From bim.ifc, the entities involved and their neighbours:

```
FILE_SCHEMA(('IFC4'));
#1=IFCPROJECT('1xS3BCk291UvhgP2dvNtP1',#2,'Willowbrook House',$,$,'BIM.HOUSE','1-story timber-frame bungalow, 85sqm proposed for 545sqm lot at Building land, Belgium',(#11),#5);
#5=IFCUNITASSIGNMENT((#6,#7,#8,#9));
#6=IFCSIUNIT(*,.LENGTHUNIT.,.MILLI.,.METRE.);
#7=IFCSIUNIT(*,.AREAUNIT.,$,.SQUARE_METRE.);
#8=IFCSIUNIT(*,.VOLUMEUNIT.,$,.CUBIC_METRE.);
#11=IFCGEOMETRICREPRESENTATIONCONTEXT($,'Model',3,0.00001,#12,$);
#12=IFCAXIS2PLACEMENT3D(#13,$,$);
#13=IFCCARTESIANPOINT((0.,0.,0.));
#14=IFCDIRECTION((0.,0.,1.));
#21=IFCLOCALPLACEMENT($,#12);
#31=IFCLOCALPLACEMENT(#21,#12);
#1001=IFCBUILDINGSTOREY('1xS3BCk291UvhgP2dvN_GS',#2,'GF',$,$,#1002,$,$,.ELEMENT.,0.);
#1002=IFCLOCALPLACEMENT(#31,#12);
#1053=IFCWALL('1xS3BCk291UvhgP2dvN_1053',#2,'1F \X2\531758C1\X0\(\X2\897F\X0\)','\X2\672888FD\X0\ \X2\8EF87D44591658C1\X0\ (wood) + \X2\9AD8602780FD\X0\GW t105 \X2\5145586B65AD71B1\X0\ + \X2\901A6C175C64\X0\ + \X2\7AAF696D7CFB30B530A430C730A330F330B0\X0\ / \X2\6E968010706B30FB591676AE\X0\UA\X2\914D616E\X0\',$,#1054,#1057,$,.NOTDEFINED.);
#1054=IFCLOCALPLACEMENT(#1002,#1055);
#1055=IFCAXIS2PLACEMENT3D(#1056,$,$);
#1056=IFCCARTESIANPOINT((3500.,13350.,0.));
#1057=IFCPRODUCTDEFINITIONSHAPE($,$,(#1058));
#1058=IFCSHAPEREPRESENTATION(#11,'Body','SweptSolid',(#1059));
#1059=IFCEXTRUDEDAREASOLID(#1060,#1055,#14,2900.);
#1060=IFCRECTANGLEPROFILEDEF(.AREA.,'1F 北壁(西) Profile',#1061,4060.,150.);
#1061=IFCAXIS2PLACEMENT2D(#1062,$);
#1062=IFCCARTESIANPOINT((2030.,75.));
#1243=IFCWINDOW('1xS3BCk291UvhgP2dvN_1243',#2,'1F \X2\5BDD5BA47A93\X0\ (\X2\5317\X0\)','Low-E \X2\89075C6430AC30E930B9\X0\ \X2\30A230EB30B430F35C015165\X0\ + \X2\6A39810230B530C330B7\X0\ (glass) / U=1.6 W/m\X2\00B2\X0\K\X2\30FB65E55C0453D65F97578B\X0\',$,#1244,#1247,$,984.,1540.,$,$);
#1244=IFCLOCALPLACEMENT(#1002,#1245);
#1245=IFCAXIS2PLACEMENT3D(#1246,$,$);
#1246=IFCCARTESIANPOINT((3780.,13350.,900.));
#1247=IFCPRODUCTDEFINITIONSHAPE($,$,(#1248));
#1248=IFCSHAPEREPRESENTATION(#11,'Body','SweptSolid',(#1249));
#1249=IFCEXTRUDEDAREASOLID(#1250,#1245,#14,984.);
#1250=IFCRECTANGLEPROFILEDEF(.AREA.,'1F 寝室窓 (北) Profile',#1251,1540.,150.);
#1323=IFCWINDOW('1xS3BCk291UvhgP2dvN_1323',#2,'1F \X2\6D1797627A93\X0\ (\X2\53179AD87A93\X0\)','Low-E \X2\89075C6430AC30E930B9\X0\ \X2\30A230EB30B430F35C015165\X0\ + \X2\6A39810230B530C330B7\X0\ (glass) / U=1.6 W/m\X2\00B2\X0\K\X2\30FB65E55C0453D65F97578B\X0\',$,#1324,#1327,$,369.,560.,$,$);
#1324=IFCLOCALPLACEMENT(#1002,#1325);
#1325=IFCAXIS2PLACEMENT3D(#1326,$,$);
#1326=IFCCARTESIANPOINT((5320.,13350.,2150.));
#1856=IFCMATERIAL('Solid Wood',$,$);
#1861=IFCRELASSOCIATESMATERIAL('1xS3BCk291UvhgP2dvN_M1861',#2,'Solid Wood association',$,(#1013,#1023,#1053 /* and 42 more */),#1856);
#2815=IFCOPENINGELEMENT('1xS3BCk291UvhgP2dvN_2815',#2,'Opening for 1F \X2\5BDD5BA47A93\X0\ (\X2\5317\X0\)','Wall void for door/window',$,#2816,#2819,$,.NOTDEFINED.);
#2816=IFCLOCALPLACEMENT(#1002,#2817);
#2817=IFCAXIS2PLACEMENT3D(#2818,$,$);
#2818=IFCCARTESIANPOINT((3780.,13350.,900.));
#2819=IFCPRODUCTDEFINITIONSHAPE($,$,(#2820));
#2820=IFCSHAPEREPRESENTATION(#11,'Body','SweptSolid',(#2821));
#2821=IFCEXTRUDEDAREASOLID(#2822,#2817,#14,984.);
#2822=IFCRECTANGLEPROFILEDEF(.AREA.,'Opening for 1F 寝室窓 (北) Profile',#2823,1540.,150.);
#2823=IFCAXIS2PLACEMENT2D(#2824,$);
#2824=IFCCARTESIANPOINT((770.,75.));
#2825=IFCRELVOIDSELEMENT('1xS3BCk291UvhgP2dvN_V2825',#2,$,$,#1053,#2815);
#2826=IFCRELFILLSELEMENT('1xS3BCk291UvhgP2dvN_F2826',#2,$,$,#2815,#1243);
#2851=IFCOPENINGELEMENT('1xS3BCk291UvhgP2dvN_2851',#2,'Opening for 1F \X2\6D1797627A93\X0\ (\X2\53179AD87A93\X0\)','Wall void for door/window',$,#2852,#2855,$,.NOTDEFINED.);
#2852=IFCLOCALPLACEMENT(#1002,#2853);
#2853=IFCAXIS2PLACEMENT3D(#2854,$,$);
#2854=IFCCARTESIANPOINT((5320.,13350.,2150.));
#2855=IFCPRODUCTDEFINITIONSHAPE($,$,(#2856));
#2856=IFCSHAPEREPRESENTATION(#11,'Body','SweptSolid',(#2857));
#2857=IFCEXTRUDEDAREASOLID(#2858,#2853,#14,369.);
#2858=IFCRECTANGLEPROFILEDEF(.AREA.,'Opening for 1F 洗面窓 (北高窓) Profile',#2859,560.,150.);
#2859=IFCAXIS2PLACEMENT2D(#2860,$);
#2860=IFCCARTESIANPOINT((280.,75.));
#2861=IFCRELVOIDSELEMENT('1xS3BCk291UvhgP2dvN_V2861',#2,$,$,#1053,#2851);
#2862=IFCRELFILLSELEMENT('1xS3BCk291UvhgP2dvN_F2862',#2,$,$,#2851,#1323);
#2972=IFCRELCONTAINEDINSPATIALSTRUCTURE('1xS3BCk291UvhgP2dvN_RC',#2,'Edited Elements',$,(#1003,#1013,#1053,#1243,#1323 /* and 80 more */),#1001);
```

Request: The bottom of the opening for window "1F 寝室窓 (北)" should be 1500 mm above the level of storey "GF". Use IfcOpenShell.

```python
import numpy as np
import ifcopenshell
import ifcopenshell.api.geometry
import ifcopenshell.geom
import ifcopenshell.util.element
import ifcopenshell.util.placement
import ifcopenshell.util.shape
import ifcopenshell.util.unit

model = ifcopenshell.open("bim.ifc")
unit_scale = ifcopenshell.util.unit.calculate_unit_scale(model)

window = model.by_id(1243)
opening = window.FillsVoids[0].RelatingOpeningElement
storey = ifcopenshell.util.element.get_container(window, ifc_class="IfcBuildingStorey")
level = ifcopenshell.util.placement.get_local_placement(storey.ObjectPlacement)[2, 3]

# The opening's origin need not be at the sill, so measure its lowest point.
shape = ifcopenshell.geom.create_shape(ifcopenshell.geom.settings(), opening)
bottom = ifcopenshell.util.shape.get_shape_bottom_elevation(shape, shape.geometry) / unit_scale
dz = level + 1500.0 - bottom

shift = np.array([0.0, 0.0, dz])
# The window is not placed relative to its opening, so move both.
for product in (opening, window):
    matrix = ifcopenshell.util.placement.get_local_placement(product.ObjectPlacement)
    matrix[:3, 3] += shift
    ifcopenshell.api.geometry.edit_object_placement(model, product=product, matrix=matrix, is_si=False)

print(f"moved by {dz * unit_scale:+.3f} m")

model.write("bim_edited.ifc")
```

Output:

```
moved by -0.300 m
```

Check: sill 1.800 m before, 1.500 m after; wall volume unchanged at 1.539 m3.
